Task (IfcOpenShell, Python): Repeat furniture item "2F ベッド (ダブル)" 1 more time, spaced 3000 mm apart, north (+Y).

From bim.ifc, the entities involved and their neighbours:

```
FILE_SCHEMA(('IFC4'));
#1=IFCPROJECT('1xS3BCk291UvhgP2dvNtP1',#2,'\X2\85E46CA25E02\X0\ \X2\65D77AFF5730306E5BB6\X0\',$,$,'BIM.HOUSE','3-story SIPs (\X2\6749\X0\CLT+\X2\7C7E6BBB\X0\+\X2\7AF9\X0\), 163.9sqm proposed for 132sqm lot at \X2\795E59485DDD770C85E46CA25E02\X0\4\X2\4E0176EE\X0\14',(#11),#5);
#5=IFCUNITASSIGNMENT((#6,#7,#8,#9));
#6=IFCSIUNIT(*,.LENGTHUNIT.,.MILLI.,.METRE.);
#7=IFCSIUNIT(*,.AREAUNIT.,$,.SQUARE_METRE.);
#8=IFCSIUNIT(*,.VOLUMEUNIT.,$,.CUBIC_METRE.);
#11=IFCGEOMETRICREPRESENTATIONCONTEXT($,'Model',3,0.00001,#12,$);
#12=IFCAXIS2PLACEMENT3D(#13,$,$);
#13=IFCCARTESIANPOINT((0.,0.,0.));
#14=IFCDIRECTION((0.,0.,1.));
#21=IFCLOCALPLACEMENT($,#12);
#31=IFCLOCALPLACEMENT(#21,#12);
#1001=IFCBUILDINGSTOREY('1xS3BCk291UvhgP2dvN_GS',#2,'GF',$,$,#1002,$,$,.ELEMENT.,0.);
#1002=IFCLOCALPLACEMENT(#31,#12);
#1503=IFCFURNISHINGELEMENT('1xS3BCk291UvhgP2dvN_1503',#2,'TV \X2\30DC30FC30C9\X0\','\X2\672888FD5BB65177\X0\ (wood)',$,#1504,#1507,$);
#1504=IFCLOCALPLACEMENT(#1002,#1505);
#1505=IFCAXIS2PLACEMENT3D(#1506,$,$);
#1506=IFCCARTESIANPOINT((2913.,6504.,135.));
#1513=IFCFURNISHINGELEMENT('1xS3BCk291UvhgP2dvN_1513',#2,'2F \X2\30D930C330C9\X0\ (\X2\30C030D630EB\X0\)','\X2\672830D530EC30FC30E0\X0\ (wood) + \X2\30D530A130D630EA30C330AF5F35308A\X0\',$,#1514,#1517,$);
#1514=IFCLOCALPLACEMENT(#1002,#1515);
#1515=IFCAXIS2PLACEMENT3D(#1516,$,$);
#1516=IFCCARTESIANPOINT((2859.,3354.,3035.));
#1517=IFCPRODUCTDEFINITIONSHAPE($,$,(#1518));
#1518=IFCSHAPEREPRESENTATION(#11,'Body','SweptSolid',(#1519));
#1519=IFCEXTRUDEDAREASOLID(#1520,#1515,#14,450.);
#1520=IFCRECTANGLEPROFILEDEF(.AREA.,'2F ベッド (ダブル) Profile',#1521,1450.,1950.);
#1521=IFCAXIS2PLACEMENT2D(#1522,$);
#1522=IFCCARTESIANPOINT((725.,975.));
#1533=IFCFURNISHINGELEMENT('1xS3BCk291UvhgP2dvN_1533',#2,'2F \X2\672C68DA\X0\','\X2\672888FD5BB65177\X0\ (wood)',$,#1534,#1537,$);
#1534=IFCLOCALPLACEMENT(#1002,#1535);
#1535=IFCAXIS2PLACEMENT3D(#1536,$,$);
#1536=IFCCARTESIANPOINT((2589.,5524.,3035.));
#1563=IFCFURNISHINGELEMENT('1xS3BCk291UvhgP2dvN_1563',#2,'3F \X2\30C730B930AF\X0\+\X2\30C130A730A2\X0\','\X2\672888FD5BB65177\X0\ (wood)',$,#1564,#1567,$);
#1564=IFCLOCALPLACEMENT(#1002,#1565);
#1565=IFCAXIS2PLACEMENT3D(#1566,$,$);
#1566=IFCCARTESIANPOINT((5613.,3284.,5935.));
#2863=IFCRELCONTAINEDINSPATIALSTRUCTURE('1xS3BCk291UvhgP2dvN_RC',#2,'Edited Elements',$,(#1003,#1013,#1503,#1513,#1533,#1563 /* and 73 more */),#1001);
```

```python
import numpy as np
import ifcopenshell
import ifcopenshell.api.geometry
import ifcopenshell.api.root
import ifcopenshell.util.element
import ifcopenshell.util.placement
import ifcopenshell.util.unit

model = ifcopenshell.open("bim.ifc")
unit_scale = ifcopenshell.util.unit.calculate_unit_scale(model)


def reuse_history(source, copy):
    """copy_class also copies each property set's owner history, people and application; keep the originals."""
    for rel in copy.IsDefinedBy:
        if rel.is_a("IfcRelDefinesByProperties") and (history := rel.RelatingPropertyDefinition.OwnerHistory):
            rel.RelatingPropertyDefinition.OwnerHistory = source.OwnerHistory
            ifcopenshell.util.element.remove_deep2(model, history)


source = model.by_id(1513)
base = ifcopenshell.util.placement.get_local_placement(source.ObjectPlacement)
step = np.array([0.0, 1.0, 0.0]) * 3 / unit_scale

for i in range(1, 2):
    copy = ifcopenshell.api.root.copy_class(model, product=source)
    copy.Representation = ifcopenshell.util.element.copy_deep(
        model, source.Representation, exclude=["IfcGeometricRepresentationContext", "IfcRepresentationMap"]
    )
    reuse_history(source, copy)
    matrix = base.copy()
    matrix[:3, 3] += i * step
    print("added at", matrix[:3, 3].round(3) + 0.0)
    ifcopenshell.api.geometry.edit_object_placement(model, product=copy, matrix=matrix, is_si=False)

model.write("bim_rev.ifc")
```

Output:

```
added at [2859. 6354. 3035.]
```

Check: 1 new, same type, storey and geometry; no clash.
